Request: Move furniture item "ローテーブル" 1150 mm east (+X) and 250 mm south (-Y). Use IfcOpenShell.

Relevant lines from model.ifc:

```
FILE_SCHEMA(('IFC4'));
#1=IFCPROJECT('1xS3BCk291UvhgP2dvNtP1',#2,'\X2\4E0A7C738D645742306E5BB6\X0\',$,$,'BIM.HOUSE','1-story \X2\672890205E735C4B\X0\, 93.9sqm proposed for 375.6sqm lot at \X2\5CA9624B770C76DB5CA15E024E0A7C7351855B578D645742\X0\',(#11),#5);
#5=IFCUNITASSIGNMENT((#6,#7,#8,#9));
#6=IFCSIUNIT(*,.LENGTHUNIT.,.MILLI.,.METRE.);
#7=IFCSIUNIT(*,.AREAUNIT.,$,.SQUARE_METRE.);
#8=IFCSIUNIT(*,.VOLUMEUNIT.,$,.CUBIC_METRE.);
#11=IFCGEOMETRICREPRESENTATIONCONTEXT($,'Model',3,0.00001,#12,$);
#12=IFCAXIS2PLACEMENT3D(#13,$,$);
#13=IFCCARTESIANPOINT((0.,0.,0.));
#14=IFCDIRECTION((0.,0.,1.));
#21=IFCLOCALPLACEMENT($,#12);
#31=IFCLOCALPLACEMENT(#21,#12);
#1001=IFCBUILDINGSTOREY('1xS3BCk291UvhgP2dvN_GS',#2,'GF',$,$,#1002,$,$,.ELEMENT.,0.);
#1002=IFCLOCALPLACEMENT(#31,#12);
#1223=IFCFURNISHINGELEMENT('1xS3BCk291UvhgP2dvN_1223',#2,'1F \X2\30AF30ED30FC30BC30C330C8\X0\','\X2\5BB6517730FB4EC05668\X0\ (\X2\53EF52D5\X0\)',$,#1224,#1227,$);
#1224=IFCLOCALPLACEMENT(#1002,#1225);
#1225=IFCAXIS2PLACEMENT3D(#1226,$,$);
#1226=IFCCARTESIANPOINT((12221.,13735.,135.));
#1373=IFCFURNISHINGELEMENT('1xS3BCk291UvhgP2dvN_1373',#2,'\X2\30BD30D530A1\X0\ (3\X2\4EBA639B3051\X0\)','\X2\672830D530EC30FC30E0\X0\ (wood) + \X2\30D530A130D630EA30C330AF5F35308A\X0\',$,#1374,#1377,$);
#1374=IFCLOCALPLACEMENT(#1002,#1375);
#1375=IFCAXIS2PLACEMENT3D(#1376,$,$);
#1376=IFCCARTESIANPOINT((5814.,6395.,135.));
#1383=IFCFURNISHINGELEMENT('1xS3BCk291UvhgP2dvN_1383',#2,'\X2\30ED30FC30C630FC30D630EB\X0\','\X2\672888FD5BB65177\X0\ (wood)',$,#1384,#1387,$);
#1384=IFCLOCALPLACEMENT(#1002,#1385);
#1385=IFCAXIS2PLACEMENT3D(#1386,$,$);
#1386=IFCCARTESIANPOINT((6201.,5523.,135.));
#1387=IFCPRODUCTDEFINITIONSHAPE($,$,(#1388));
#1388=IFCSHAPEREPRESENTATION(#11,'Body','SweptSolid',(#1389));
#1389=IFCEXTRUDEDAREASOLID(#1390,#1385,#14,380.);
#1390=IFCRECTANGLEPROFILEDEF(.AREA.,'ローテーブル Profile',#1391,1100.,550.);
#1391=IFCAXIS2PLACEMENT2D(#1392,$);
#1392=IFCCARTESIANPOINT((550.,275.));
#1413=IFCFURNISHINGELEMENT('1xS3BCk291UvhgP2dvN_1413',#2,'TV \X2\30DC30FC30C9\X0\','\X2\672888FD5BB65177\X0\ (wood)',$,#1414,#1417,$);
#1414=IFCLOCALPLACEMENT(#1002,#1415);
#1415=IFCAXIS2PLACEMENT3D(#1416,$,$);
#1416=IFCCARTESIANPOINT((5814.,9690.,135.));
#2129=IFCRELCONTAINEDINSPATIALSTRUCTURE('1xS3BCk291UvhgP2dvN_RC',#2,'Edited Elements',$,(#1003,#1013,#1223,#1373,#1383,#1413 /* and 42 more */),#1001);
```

```python
import ifcopenshell
import ifcopenshell.api.geometry
import ifcopenshell.util.placement
import ifcopenshell.util.unit

model = ifcopenshell.open("model.ifc")
unit_scale = ifcopenshell.util.unit.calculate_unit_scale(model)

item = model.by_guid("1xS3BCk291UvhgP2dvN_1383")
matrix = ifcopenshell.util.placement.get_local_placement(item.ObjectPlacement)
matrix[0, 3] += 1.15 / unit_scale
matrix[1, 3] -= 0.25 / unit_scale
ifcopenshell.api.geometry.edit_object_placement(model, product=item, matrix=matrix, is_si=False)

print(ifcopenshell.util.placement.get_local_placement(item.ObjectPlacement).round(3) + 0.0)

model.write("model_updated.ifc")
```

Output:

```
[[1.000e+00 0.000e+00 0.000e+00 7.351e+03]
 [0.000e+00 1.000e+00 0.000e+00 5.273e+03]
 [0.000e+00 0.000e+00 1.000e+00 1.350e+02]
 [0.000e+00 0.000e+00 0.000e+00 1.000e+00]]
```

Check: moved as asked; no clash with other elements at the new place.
